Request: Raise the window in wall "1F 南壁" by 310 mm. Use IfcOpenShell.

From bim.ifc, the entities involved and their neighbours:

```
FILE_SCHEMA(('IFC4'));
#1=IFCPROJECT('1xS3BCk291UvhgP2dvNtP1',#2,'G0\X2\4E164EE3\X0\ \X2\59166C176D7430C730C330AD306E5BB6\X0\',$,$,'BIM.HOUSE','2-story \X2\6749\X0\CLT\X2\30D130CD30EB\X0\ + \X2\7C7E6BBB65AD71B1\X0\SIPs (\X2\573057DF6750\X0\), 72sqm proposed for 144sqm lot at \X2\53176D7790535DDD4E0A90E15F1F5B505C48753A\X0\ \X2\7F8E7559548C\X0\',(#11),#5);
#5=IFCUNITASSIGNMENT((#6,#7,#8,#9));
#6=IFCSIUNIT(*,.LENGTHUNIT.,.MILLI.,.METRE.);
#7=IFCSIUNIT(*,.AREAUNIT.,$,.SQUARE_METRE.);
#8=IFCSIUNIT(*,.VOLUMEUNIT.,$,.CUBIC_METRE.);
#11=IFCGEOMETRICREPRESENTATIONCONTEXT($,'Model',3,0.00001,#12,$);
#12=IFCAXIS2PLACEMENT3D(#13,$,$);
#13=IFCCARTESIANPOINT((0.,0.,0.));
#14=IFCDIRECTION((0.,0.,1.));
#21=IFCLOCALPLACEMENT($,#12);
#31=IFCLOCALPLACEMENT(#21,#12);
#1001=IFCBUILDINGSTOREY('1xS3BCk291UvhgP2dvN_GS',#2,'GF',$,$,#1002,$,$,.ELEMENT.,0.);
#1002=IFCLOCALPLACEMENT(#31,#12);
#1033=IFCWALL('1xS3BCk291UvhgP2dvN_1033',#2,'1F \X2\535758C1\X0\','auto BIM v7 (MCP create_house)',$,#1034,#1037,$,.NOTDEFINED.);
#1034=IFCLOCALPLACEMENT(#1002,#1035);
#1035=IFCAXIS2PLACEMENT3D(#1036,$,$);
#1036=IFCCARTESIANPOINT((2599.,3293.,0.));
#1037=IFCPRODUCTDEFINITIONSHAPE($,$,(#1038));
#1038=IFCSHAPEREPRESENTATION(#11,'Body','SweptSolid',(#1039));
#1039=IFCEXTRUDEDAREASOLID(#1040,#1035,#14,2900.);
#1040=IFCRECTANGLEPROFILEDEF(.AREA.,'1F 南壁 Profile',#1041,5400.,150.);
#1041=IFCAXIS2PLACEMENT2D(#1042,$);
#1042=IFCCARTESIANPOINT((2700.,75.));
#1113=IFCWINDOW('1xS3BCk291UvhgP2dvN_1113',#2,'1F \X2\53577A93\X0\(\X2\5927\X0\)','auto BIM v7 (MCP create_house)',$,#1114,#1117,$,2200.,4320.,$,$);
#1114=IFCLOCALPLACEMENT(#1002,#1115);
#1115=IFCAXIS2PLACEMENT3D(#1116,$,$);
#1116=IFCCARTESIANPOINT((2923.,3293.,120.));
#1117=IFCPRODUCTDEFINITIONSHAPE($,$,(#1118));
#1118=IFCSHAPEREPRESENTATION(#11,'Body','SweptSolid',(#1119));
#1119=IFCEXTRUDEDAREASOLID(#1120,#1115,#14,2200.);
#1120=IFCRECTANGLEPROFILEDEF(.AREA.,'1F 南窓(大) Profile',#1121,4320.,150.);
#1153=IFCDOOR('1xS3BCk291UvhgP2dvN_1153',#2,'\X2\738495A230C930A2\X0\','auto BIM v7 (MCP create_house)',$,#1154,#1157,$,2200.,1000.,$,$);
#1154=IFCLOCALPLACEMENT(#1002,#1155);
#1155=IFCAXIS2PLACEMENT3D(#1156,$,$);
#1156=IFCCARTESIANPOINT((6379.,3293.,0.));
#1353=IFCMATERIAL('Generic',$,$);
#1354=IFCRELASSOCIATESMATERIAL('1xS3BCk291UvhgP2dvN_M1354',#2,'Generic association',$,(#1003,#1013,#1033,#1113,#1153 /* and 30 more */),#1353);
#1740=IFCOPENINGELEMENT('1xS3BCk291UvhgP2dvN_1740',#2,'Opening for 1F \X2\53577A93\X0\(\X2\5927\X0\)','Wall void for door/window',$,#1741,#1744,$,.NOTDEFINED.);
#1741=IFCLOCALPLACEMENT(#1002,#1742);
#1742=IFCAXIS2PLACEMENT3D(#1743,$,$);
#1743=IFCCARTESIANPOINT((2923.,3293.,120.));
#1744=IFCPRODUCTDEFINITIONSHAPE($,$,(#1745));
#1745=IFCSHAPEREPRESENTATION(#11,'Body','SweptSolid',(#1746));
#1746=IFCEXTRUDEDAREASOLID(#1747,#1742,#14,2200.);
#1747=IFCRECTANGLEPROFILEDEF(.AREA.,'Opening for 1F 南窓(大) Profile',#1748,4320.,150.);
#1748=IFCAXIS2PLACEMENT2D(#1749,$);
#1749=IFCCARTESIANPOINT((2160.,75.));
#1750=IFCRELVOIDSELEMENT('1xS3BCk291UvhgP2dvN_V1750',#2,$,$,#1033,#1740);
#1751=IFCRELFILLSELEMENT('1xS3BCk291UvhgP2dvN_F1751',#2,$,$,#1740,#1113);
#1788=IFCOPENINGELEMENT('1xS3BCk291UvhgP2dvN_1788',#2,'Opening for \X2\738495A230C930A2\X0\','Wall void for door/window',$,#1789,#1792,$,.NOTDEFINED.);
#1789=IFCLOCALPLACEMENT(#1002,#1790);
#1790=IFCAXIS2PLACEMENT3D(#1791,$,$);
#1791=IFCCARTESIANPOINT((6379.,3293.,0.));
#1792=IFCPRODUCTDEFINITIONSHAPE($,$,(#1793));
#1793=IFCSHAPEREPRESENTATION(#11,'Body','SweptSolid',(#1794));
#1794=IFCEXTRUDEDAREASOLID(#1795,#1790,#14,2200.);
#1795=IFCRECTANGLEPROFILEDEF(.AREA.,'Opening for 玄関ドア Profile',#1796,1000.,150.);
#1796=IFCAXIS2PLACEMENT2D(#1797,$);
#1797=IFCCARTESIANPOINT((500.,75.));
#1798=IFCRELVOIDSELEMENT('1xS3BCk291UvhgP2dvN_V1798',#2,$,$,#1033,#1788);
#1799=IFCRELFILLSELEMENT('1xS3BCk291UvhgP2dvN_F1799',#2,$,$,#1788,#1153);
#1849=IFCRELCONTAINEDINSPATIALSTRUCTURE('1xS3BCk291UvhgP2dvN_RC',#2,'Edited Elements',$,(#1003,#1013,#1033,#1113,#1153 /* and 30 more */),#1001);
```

```python
import numpy as np
import ifcopenshell
import ifcopenshell.api.geometry
import ifcopenshell.util.placement
import ifcopenshell.util.unit

model = ifcopenshell.open("bim.ifc")
unit_scale = ifcopenshell.util.unit.calculate_unit_scale(model)

window = model.by_guid("1xS3BCk291UvhgP2dvN_1113")
opening = window.FillsVoids[0].RelatingOpeningElement
dz = 310.0

shift = np.array([0.0, 0.0, dz])
# The window is not placed relative to its opening, so move both.
for product in (opening, window):
    matrix = ifcopenshell.util.placement.get_local_placement(product.ObjectPlacement)
    matrix[:3, 3] += shift
    ifcopenshell.api.geometry.edit_object_placement(model, product=product, matrix=matrix, is_si=False)

print(f"moved by {dz * unit_scale:+.3f} m")

model.write("bim_edited.ifc")
```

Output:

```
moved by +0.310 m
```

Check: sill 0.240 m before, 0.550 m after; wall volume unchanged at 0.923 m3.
